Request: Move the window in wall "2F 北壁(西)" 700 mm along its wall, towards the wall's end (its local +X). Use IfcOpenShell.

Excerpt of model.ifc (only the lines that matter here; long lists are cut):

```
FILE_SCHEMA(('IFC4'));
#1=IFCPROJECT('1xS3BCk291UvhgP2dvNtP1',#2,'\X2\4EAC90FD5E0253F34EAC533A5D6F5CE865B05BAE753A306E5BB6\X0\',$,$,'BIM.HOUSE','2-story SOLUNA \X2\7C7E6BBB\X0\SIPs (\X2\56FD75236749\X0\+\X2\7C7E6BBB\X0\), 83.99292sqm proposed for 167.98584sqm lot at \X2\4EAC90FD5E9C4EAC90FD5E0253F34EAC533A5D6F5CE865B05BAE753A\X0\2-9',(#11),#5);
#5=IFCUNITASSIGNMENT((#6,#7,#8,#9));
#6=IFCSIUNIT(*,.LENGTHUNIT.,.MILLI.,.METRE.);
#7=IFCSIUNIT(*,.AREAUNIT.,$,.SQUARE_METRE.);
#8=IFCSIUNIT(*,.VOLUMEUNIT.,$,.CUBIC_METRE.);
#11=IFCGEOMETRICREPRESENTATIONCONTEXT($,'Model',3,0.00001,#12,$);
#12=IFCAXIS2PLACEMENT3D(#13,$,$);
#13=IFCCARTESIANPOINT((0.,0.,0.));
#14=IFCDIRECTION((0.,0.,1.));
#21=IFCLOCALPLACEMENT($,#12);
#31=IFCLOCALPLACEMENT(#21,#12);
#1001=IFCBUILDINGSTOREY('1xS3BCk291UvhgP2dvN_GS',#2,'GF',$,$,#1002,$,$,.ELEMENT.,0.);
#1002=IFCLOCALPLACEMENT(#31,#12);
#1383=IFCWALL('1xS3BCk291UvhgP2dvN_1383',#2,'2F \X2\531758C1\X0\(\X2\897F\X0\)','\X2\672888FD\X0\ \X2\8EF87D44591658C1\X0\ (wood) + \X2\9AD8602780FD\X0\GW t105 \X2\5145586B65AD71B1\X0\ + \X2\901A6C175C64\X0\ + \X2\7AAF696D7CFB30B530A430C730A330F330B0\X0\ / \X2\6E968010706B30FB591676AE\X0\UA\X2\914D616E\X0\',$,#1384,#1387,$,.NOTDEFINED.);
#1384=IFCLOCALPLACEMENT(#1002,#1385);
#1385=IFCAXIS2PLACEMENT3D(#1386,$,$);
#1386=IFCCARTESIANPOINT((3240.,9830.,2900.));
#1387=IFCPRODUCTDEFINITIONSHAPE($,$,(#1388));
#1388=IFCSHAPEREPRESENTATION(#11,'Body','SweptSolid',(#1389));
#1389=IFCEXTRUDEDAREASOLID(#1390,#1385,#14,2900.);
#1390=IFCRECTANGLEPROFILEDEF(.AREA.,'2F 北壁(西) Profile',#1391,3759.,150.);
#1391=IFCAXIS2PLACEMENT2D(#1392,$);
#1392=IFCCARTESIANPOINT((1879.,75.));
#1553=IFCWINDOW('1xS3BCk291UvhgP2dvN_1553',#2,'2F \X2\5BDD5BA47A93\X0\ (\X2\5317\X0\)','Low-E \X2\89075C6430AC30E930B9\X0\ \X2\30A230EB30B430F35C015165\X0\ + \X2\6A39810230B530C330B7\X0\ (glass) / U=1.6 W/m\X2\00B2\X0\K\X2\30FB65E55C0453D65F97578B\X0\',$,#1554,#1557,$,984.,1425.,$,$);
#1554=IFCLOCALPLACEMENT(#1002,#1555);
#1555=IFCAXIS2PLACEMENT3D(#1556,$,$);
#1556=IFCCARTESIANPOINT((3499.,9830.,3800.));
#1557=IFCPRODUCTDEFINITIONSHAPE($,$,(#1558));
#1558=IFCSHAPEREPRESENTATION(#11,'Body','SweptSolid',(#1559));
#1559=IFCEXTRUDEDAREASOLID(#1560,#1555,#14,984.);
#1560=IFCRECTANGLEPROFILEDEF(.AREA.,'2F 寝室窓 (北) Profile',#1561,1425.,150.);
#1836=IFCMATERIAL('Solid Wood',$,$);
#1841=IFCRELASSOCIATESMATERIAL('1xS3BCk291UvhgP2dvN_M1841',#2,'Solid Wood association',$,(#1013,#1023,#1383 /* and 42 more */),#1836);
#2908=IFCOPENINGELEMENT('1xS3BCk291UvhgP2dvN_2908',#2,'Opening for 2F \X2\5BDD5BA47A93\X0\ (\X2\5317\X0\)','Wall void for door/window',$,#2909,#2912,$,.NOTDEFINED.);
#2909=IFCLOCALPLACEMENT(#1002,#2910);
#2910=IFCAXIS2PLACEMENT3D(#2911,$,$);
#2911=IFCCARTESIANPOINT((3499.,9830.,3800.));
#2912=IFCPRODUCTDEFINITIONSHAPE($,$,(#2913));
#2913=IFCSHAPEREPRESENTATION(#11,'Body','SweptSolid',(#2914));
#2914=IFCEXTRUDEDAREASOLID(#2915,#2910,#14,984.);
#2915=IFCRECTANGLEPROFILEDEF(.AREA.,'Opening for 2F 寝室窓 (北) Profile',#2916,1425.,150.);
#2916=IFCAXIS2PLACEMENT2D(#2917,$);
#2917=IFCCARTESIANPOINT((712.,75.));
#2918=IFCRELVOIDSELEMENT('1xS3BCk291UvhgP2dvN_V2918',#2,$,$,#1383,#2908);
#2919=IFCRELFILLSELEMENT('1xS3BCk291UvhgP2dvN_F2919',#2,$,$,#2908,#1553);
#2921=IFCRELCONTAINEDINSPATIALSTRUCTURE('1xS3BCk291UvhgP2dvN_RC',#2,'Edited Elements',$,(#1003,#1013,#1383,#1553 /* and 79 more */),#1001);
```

```python
import ifcopenshell
import ifcopenshell.api.geometry
import ifcopenshell.util.placement
import ifcopenshell.util.unit

model = ifcopenshell.open("model.ifc")
unit_scale = ifcopenshell.util.unit.calculate_unit_scale(model)

window = model.by_id(1553)
opening = window.FillsVoids[0].RelatingOpeningElement
wall = opening.VoidsElements[0].RelatingBuildingElement

wall_matrix = ifcopenshell.util.placement.get_local_placement(wall.ObjectPlacement)
shift = wall_matrix[:3, 0] * 0.7 / unit_scale
before = ifcopenshell.util.placement.get_local_placement(window.ObjectPlacement)[:3, 3].copy()

# The window is not placed relative to its opening, so move both.
for product in (opening, window):
    matrix = ifcopenshell.util.placement.get_local_placement(product.ObjectPlacement)
    matrix[:3, 3] += shift
    ifcopenshell.api.geometry.edit_object_placement(model, product=product, matrix=matrix, is_si=False)

after = ifcopenshell.util.placement.get_local_placement(window.ObjectPlacement)[:3, 3]
print("window moved by", (after - before).round(3) + 0.0)

model.write("model_updated.ifc")
```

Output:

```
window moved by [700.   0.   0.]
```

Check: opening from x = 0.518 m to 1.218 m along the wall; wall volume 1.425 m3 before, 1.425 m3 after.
